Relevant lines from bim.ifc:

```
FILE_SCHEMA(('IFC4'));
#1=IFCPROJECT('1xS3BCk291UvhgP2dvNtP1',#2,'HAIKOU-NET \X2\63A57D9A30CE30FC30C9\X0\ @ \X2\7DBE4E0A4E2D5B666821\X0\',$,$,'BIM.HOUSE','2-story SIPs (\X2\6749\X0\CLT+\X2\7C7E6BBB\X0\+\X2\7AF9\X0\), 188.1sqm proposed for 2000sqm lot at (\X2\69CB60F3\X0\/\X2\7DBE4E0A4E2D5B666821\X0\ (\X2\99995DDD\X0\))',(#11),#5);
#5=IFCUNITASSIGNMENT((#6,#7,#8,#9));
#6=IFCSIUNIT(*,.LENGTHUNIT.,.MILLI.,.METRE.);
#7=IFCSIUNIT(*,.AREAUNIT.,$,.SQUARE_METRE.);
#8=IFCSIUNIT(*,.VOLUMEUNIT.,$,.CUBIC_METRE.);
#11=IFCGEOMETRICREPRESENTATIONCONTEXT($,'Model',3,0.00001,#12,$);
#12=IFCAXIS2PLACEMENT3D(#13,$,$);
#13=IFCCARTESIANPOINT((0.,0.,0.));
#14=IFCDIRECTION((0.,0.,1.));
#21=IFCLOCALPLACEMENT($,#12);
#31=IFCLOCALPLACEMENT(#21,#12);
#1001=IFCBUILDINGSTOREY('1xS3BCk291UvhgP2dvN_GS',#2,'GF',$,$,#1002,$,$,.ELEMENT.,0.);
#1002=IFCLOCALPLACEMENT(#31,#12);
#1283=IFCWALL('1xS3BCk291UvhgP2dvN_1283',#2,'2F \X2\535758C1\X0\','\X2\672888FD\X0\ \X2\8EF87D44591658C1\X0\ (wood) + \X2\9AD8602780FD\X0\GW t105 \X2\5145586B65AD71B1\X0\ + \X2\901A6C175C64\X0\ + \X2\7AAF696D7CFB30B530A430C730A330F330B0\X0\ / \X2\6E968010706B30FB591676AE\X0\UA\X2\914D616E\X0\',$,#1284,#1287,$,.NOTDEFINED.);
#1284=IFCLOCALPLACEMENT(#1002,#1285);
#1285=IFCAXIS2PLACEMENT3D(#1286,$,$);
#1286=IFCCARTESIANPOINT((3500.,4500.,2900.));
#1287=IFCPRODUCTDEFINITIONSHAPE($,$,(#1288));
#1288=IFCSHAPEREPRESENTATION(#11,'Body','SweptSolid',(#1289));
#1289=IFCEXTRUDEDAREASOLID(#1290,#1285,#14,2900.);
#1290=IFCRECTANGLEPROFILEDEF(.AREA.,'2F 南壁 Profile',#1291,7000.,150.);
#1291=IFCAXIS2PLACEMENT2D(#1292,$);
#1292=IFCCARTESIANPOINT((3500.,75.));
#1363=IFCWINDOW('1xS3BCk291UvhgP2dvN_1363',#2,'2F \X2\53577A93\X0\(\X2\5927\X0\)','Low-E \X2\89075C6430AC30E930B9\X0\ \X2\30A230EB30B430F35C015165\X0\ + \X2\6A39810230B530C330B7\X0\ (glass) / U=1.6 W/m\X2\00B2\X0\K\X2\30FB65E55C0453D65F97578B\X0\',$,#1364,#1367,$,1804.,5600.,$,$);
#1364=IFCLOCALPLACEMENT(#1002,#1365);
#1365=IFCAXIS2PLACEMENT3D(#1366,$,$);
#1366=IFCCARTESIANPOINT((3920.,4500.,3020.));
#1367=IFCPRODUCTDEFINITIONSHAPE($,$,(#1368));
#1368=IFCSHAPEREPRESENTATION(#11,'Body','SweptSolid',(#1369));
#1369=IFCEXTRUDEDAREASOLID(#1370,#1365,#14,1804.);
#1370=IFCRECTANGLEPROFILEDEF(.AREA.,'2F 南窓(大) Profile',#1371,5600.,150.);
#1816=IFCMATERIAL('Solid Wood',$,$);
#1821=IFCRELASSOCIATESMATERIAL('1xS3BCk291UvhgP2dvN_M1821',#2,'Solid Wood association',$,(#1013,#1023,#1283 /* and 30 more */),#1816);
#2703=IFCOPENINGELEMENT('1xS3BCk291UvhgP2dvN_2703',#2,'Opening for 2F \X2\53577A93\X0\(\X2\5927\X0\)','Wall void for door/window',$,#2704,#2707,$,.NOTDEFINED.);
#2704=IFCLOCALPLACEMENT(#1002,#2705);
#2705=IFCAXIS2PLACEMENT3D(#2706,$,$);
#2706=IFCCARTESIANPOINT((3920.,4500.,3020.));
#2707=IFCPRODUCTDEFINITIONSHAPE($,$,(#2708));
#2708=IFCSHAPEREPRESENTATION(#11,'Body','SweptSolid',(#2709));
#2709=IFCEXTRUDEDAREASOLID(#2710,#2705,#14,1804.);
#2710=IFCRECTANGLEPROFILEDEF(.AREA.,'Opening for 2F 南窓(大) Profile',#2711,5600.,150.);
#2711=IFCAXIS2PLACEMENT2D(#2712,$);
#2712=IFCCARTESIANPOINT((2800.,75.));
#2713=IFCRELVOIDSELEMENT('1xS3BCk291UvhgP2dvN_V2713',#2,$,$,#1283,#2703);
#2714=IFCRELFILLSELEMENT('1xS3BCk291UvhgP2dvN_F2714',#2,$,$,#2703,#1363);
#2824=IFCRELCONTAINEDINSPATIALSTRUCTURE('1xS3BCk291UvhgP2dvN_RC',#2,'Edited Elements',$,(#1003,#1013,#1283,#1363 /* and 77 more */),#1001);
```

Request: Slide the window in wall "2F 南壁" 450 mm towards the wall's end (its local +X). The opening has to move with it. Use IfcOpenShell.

```python
import ifcopenshell
import ifcopenshell.api.geometry
import ifcopenshell.util.placement

model = ifcopenshell.open("bim.ifc")

window = model.by_guid("1xS3BCk291UvhgP2dvN_1363")
opening = window.FillsVoids[0].RelatingOpeningElement
wall = opening.VoidsElements[0].RelatingBuildingElement

wall_matrix = ifcopenshell.util.placement.get_local_placement(wall.ObjectPlacement)
shift = wall_matrix[:3, 0] * 450.0
before = ifcopenshell.util.placement.get_local_placement(window.ObjectPlacement)[:3, 3].copy()

# The window is not placed relative to its opening, so move both.
for product in (opening, window):
    matrix = ifcopenshell.util.placement.get_local_placement(product.ObjectPlacement)
    matrix[:3, 3] += shift
    ifcopenshell.api.geometry.edit_object_placement(model, product=product, matrix=matrix, is_si=False)

after = ifcopenshell.util.placement.get_local_placement(window.ObjectPlacement)[:3, 3]
print("window moved by", (after - before).round(3) + 0.0)

model.write("bim_updated.ifc")
```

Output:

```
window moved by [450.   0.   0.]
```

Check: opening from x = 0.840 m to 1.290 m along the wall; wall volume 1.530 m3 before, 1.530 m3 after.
